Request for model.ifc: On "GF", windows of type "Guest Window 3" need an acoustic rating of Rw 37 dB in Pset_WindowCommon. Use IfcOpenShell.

First a look at what the model holds.

```python
import ifcopenshell
import ifcopenshell.util.element

model = ifcopenshell.open("model.ifc")
print(model.schema)
storey = next(s for s in model.by_type("IfcBuildingStorey") if s.Name == "GF")
windows = [e for e in ifcopenshell.util.element.get_decomposition(storey) if e.is_a("IfcWindow")]
seen = {}
for e in windows:
    element_type = ifcopenshell.util.element.get_type(e)
    key = (element_type.Name if element_type != e and element_type else None, ifcopenshell.util.element.get_pset(e, "Pset_WindowCommon", "AcousticRating"))
    seen[key] = seen.get(key, 0) + 1
for (name, value), count in sorted(seen.items(), key=str):
    print(count, "x", name, "|", value)
```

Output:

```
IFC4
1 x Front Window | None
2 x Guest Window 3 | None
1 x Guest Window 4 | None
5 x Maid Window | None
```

```python
import ifcopenshell
import ifcopenshell.api.pset
import ifcopenshell.util.element

model = ifcopenshell.open("model.ifc")

storey = next(s for s in model.by_type("IfcBuildingStorey") if s.Name == "GF")
windows = [e for e in ifcopenshell.util.element.get_decomposition(storey) if e.is_a("IfcWindow")]

count = 0
for e in windows:
    element_type = ifcopenshell.util.element.get_type(e)
    if element_type in (None, e) or element_type.Name != "Guest Window 3":
        continue
    # add_pset returns the element's existing set when there is one.
    pset = ifcopenshell.api.pset.add_pset(model, product=e, name="Pset_WindowCommon")
    ifcopenshell.api.pset.edit_pset(model, pset=pset, properties={"AcousticRating": "Rw 37 dB"})
    count += 1

print(count, "windows updated")

model.write("model_updated.ifc")
```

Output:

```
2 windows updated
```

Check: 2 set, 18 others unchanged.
